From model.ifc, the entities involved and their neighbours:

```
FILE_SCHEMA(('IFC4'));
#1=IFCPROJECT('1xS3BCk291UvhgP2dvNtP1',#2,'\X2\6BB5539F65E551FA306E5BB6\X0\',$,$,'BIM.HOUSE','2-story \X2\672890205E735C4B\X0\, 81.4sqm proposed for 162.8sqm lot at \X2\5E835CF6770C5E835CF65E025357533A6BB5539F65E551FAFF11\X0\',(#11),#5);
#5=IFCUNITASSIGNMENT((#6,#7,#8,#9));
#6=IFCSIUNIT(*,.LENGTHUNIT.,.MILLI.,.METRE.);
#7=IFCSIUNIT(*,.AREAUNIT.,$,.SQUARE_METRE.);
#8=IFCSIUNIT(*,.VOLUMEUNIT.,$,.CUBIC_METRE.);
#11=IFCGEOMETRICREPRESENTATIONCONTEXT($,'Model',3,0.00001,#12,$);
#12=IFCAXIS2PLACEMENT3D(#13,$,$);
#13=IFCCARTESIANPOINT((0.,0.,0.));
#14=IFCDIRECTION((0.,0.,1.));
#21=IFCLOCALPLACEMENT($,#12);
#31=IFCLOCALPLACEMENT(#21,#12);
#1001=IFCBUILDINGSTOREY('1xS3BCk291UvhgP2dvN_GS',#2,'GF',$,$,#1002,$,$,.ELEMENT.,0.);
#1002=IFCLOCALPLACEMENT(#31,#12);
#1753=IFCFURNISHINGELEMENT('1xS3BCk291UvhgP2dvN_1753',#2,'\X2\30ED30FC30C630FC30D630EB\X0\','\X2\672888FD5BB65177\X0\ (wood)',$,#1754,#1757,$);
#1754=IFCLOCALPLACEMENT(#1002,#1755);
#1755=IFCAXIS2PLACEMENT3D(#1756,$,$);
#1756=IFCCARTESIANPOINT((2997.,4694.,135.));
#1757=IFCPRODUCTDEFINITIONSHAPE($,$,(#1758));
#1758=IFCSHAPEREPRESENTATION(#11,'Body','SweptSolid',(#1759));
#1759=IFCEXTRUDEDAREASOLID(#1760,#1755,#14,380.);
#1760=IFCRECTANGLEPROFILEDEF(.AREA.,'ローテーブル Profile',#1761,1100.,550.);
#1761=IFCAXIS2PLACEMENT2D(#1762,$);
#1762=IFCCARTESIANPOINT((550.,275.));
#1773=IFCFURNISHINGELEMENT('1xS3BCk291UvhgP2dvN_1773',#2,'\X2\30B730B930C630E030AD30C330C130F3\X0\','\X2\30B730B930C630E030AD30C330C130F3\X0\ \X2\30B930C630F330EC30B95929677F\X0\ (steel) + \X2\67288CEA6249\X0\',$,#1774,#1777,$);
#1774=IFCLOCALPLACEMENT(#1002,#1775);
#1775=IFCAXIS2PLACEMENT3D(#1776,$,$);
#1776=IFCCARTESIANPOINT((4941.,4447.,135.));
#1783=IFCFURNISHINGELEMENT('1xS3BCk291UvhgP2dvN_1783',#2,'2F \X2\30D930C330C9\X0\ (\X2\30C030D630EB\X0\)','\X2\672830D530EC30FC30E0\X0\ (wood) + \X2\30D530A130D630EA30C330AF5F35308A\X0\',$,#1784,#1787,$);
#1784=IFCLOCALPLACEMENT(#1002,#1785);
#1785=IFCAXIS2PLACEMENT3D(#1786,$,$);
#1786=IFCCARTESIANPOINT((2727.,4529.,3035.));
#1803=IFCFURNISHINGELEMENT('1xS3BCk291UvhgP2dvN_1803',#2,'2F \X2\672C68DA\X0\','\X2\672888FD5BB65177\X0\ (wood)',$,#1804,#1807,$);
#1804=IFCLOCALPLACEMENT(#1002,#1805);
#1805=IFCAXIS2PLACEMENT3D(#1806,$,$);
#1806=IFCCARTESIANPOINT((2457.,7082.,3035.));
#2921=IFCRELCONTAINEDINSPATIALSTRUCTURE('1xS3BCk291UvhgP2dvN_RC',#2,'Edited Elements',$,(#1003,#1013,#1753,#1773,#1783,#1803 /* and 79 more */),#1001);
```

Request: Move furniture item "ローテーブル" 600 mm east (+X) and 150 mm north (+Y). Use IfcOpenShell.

```python
import ifcopenshell
import ifcopenshell.api.geometry
import ifcopenshell.util.placement
import ifcopenshell.util.unit

model = ifcopenshell.open("model.ifc")
unit_scale = ifcopenshell.util.unit.calculate_unit_scale(model)

item = model.by_guid("1xS3BCk291UvhgP2dvN_1753")
matrix = ifcopenshell.util.placement.get_local_placement(item.ObjectPlacement)
matrix[0, 3] += 0.6 / unit_scale
matrix[1, 3] += 0.15 / unit_scale
ifcopenshell.api.geometry.edit_object_placement(model, product=item, matrix=matrix, is_si=False)

print(ifcopenshell.util.placement.get_local_placement(item.ObjectPlacement).round(3) + 0.0)

model.write("model_updated.ifc")
```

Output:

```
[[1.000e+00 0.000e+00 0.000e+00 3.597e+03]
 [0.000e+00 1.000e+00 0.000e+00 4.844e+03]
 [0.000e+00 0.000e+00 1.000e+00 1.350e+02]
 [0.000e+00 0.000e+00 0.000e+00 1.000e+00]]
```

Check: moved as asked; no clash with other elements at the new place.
